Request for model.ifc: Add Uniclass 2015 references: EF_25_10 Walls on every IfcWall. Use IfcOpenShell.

First a look at what the model holds.

```python
import ifcopenshell

model = ifcopenshell.open("model.ifc")
print(model.schema)
print("classifications:", [c.Name for c in model.by_type("IfcClassification")])
for ifc_class in ("IfcDoor", "IfcRoof", "IfcStair", "IfcWall", "IfcWindow"):
    print(ifc_class, len(model.by_type(ifc_class)))
```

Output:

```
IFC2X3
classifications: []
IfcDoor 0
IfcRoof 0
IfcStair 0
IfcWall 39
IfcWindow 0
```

```python
import ifcopenshell
import ifcopenshell.api.classification

model = ifcopenshell.open("model.ifc")

# IFC2X3 requires Source and Edition and has no link from the project to the system.
system = model.create_entity("IfcClassification", Source="NBS", Edition="2015", Name="Uniclass 2015")

codes = {
    "IfcWall": ("EF_25_10", "Walls"),
}
for ifc_class, (code, name) in codes.items():
    products = model.by_type(ifc_class)
    ifcopenshell.api.classification.add_reference(
        model, products=products, classification=system, identification=code, name=name
    )
    print(code, len(products))

model.write("model_updated.ifc")
```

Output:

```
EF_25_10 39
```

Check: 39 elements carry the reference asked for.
